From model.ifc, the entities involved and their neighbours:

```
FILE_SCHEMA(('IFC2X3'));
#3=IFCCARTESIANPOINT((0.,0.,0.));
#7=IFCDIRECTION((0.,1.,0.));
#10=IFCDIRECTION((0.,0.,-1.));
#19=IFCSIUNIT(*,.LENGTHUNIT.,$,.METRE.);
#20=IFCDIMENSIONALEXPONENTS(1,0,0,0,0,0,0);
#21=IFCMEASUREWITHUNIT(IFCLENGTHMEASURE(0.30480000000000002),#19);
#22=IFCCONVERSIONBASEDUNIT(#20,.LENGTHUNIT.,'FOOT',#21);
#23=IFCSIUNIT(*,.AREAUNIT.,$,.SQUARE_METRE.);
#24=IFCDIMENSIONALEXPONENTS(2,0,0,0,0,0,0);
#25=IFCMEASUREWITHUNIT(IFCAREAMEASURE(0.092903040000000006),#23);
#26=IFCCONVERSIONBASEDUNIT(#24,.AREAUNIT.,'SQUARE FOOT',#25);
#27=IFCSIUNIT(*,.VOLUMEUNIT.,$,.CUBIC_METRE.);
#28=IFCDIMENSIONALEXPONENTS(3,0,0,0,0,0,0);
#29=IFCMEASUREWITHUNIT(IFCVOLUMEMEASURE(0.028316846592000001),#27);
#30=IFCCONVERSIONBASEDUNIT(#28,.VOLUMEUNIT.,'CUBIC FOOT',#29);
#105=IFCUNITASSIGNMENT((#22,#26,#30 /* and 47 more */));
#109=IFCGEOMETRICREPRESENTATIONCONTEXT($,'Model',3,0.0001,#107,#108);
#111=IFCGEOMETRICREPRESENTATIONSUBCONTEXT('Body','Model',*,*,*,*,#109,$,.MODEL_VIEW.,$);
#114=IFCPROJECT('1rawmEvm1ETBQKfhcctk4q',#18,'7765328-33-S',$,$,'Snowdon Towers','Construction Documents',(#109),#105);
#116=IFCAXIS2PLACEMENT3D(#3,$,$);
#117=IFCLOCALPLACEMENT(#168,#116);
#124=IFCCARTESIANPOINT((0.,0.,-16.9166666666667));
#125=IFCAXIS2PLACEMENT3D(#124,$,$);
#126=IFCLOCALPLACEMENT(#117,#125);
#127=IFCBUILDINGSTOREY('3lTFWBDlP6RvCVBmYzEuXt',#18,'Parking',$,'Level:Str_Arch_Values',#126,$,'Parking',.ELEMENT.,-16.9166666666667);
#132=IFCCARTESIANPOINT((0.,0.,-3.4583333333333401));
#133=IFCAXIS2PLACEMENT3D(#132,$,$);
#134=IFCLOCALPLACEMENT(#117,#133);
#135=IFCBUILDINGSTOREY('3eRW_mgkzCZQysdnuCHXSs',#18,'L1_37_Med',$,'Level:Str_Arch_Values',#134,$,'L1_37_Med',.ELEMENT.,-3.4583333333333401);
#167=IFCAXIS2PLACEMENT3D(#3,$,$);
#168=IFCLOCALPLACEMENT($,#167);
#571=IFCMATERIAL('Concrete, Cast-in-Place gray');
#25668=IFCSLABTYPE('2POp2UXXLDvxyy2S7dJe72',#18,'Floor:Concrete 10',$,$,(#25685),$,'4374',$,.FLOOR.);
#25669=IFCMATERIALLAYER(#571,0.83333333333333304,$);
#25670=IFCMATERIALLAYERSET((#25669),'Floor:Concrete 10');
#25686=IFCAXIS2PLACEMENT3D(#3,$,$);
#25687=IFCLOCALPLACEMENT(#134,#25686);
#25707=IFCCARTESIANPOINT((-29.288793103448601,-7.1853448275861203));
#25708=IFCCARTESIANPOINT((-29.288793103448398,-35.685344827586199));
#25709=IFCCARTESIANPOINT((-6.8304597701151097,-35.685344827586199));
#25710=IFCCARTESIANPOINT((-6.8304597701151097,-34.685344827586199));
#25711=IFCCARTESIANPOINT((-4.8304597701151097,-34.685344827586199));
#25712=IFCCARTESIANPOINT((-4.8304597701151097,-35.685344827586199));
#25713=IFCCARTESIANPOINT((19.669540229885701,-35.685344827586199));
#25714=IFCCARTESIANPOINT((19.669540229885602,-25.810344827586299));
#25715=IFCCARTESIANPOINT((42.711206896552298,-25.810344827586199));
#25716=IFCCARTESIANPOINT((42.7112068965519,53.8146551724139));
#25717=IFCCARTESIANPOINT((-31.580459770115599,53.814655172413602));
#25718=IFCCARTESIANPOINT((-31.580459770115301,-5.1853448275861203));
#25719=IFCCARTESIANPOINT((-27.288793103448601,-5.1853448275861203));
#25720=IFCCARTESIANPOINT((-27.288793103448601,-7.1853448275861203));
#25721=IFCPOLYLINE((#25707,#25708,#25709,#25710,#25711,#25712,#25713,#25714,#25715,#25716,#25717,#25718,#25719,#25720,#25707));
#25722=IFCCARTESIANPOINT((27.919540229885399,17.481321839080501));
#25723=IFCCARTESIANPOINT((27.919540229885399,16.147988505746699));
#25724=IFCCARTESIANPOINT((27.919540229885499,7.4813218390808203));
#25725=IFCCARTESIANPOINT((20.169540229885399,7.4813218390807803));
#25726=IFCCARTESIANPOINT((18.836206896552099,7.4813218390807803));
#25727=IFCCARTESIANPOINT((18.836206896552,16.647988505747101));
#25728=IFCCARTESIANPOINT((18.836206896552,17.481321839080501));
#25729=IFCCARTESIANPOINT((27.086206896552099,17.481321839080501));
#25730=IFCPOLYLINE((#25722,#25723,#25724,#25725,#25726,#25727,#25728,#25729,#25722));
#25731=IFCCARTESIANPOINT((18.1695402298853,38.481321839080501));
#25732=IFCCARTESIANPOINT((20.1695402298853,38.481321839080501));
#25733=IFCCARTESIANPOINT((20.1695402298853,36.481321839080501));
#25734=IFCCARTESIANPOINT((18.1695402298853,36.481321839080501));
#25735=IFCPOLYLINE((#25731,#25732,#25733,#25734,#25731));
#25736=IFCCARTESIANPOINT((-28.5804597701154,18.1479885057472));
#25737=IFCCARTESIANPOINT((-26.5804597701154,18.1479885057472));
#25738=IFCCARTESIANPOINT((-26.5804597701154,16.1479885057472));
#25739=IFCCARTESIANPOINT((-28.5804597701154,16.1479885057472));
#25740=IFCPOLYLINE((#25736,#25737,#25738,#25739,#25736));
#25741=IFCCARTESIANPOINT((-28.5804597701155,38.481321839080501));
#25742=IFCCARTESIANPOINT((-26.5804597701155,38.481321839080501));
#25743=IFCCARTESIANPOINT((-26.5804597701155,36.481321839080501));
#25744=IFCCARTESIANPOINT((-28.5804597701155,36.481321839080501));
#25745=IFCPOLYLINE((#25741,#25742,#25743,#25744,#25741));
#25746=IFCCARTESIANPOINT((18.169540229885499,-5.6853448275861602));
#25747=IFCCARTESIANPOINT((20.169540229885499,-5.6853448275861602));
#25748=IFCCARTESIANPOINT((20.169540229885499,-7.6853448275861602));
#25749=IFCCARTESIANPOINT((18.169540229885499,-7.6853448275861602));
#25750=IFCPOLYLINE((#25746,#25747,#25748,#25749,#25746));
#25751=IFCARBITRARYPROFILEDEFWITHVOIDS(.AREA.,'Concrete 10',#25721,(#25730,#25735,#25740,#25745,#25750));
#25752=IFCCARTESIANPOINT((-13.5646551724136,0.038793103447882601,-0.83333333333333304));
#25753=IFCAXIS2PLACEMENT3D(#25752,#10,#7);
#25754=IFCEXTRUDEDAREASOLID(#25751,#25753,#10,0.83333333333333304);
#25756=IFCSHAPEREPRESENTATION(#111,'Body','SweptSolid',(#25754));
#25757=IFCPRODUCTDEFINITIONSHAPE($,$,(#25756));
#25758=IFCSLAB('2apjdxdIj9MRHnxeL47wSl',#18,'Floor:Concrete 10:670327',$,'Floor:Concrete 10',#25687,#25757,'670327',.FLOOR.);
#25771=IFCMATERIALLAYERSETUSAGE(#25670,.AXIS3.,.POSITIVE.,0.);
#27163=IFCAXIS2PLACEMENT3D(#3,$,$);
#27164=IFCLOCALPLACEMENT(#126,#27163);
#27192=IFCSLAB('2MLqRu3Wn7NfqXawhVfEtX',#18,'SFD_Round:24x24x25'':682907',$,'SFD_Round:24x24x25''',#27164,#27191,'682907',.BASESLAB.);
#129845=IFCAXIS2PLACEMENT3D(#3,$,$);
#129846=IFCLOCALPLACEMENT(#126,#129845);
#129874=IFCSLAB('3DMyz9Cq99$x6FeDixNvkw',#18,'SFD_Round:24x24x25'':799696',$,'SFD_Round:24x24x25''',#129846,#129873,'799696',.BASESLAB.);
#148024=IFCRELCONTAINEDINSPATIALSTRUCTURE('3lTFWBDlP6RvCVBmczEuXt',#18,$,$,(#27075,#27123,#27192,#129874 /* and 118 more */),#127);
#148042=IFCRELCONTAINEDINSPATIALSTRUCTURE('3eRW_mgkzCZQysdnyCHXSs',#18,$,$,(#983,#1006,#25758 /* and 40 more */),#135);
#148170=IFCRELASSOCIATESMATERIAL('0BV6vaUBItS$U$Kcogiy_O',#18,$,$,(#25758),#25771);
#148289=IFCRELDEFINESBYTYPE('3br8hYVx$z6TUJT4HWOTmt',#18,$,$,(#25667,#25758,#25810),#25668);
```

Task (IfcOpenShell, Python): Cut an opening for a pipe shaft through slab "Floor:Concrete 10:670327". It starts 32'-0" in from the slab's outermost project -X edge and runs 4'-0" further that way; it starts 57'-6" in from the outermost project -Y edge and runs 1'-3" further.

```python
import numpy as np
import ifcopenshell
import ifcopenshell.api.feature
import ifcopenshell.api.geometry
import ifcopenshell.api.root
import ifcopenshell.geom
import ifcopenshell.util.placement
import ifcopenshell.util.representation
import ifcopenshell.util.shape
import ifcopenshell.util.unit

model = ifcopenshell.open("model.ifc")
unit_scale = ifcopenshell.util.unit.calculate_unit_scale(model)
settings = ifcopenshell.geom.settings()


def volume(element):
    """Net volume in cubic metres, openings subtracted."""
    shape = ifcopenshell.geom.create_shape(settings, element)
    return ifcopenshell.util.shape.get_volume(shape.geometry)


slab = model.by_id(25758)
before = volume(slab)

# Extent in the slab's own axes, in metres. The edges named are its -X and -Y sides.
slab_shape = ifcopenshell.geom.create_shape(settings, slab)
vertices = ifcopenshell.util.shape.get_vertices(slab_shape.geometry)
x_min, y_min, bottom = vertices.min(axis=0)
top = vertices[:, 2].max()

opening = ifcopenshell.api.root.create_entity(model, ifc_class="IfcOpeningElement", name="Pipe shaft opening")
context = ifcopenshell.util.representation.get_context(model, "Model", "Body", "MODEL_VIEW")
width, depth = 1.2192, 0.381
outline = [(0.0, 0.0), (width, 0.0), (width, depth), (0.0, depth), (0.0, 0.0)]
# Overshoot both faces by 50 mm so the cut is clean.
shape = ifcopenshell.api.geometry.add_slab_representation(
    model, context=context, depth=top - bottom + 0.1, polyline=outline
)
ifcopenshell.api.geometry.assign_representation(model, product=opening, representation=shape)

matrix = ifcopenshell.util.placement.get_local_placement(slab.ObjectPlacement)
matrix[:, 3] = matrix @ np.append(np.array([x_min + 9.7536, y_min + 17.526, bottom - 0.05]) / unit_scale, 1.0)
ifcopenshell.api.geometry.edit_object_placement(model, product=opening, matrix=matrix, is_si=False)
ifcopenshell.api.feature.add_feature(model, feature=opening, element=slab)

after = volume(slab)

print(f"slab volume {before:.3f} -> {after:.3f} m3")

model.write("model_edited.ifc")
```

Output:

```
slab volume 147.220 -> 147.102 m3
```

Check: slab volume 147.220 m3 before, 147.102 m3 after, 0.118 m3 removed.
